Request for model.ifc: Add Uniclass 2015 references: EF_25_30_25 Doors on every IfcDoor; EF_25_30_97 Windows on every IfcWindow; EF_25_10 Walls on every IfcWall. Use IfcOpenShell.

First a look at what the model holds.

```python
import ifcopenshell

model = ifcopenshell.open("model.ifc")
print(model.schema)
print("classifications:", [c.Name for c in model.by_type("IfcClassification")])
for ifc_class in ("IfcDoor", "IfcRoof", "IfcStair", "IfcWall", "IfcWindow"):
    print(ifc_class, len(model.by_type(ifc_class)))
```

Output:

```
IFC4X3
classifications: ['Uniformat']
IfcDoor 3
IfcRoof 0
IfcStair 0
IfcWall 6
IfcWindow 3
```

```python
import ifcopenshell
import ifcopenshell.api.classification

model = ifcopenshell.open("model.ifc")

system = ifcopenshell.api.classification.add_classification(model, classification="Uniclass 2015")

codes = {
    "IfcDoor": ("EF_25_30_25", "Doors"),
    "IfcWindow": ("EF_25_30_97", "Windows"),
    "IfcWall": ("EF_25_10", "Walls"),
}
for ifc_class, (code, name) in codes.items():
    products = model.by_type(ifc_class)
    ifcopenshell.api.classification.add_reference(
        model, products=products, classification=system, identification=code, name=name
    )
    print(code, len(products))

model.write("model_v2.ifc")
```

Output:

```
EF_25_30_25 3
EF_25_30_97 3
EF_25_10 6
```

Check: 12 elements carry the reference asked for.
